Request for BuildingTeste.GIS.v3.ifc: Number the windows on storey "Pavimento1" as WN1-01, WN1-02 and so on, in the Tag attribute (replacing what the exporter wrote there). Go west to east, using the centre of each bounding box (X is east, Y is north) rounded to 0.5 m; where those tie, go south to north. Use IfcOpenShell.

First a look at what the model holds.

```python
import ifcopenshell
import ifcopenshell.util.element
import ifcopenshell.util.placement

model = ifcopenshell.open("BuildingTeste.GIS.v3.ifc")
print(model.schema)
storey = next(s for s in model.by_type("IfcBuildingStorey") if s.Name == "Pavimento1")
windows = [e for e in ifcopenshell.util.element.get_decomposition(storey) if e.is_a("IfcWindow")]
for e in sorted(windows, key=lambda e: e.id()):
    origin = ifcopenshell.util.placement.get_local_placement(e.ObjectPlacement)[:3, 3]
    print(e.id(), e.Tag, e.Name, origin.round(2) + 0.0, sep=" | ")
```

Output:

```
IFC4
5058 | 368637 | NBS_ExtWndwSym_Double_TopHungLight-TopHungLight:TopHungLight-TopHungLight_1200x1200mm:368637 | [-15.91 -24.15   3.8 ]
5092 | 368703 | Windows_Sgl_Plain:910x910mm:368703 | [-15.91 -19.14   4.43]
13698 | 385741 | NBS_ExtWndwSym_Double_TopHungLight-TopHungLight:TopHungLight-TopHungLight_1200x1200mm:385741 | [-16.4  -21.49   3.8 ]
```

```python
import ifcopenshell
import ifcopenshell.geom
import ifcopenshell.util.element
import ifcopenshell.util.shape

model = ifcopenshell.open("BuildingTeste.GIS.v3.ifc")
settings = ifcopenshell.geom.settings()
settings.set("use-world-coords", True)


def centre(element):
    shape = ifcopenshell.geom.create_shape(settings, element)
    return ifcopenshell.util.shape.get_bbox_centroid(shape.geometry)


storey = next(s for s in model.by_type("IfcBuildingStorey") if s.Name == "Pavimento1")
windows = [e for e in ifcopenshell.util.element.get_decomposition(storey) if e.is_a("IfcWindow")]

# Insertion points can sit at a corner or the storey origin, so sort by the geometry (in metres).
centres = {e: centre(e) for e in windows}
windows.sort(key=lambda e: (round(centres[e][0] / 0.5), centres[e][1]))

for i, e in enumerate(windows, start=1):
    number = f"WN1-{i:02d}"
    e.Tag = number
    print(e.id(), number)

model.write("BuildingTeste.GIS.v3-out.ifc")
```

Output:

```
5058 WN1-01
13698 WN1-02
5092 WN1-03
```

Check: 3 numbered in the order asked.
